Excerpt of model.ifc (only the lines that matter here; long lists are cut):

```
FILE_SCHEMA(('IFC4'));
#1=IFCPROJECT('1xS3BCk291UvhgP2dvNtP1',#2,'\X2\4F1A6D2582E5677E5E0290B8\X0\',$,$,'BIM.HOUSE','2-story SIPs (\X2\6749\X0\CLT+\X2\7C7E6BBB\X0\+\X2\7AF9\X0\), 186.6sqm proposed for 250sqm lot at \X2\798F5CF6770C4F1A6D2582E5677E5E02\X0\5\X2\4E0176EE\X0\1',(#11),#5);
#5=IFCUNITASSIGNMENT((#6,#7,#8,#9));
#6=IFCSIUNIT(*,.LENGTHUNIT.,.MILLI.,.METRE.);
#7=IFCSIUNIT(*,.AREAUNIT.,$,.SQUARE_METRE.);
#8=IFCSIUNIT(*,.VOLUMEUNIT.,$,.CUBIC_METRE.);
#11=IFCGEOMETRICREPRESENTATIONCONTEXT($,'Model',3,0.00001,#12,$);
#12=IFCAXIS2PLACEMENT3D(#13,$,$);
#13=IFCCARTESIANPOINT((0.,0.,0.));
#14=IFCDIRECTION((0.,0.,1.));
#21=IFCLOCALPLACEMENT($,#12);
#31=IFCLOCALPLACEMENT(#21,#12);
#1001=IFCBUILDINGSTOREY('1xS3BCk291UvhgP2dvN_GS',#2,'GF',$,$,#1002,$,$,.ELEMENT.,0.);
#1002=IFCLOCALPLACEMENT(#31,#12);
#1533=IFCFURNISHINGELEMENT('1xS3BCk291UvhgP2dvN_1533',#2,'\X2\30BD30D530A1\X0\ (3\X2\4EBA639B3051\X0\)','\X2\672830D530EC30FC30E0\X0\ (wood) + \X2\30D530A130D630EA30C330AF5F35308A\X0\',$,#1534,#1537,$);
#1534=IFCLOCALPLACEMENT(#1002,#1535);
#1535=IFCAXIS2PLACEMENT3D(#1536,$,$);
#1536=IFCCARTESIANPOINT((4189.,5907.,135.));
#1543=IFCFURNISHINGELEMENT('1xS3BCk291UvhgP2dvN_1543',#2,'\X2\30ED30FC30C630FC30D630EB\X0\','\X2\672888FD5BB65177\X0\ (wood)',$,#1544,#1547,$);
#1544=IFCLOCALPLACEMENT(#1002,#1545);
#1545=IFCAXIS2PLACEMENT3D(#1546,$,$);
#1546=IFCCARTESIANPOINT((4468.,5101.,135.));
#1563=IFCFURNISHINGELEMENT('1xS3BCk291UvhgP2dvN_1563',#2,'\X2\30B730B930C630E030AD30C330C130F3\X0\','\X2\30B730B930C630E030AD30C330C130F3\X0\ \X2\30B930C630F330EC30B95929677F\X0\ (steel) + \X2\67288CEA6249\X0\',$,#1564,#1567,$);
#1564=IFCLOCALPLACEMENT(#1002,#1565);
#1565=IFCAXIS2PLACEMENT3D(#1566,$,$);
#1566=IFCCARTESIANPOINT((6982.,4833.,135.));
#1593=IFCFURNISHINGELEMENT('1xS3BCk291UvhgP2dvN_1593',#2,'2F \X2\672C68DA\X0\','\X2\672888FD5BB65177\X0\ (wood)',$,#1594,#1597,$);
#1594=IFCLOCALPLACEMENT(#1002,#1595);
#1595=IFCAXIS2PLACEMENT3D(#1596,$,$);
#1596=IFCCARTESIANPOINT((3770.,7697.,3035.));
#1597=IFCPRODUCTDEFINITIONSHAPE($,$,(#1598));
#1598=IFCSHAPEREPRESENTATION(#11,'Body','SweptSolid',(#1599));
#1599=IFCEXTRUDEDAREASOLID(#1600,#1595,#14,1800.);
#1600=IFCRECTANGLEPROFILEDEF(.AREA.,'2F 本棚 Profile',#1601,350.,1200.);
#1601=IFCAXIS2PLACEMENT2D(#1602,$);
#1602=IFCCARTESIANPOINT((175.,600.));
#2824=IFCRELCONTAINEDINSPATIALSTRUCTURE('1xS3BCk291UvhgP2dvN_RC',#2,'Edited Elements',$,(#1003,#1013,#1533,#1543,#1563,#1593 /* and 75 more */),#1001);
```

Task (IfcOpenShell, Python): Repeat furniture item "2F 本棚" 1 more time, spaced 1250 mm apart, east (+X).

```python
import numpy as np
import ifcopenshell
import ifcopenshell.api.geometry
import ifcopenshell.api.root
import ifcopenshell.util.element
import ifcopenshell.util.placement
import ifcopenshell.util.unit

model = ifcopenshell.open("model.ifc")
unit_scale = ifcopenshell.util.unit.calculate_unit_scale(model)


def reuse_history(source, copy):
    """copy_class also copies each property set's owner history, people and application; keep the originals."""
    for rel in copy.IsDefinedBy:
        if rel.is_a("IfcRelDefinesByProperties") and (history := rel.RelatingPropertyDefinition.OwnerHistory):
            rel.RelatingPropertyDefinition.OwnerHistory = source.OwnerHistory
            ifcopenshell.util.element.remove_deep2(model, history)


source = model.by_id(1593)
base = ifcopenshell.util.placement.get_local_placement(source.ObjectPlacement)
step = np.array([1.0, 0.0, 0.0]) * 1.25 / unit_scale

for i in range(1, 2):
    copy = ifcopenshell.api.root.copy_class(model, product=source)
    copy.Representation = ifcopenshell.util.element.copy_deep(
        model, source.Representation, exclude=["IfcGeometricRepresentationContext", "IfcRepresentationMap"]
    )
    reuse_history(source, copy)
    matrix = base.copy()
    matrix[:3, 3] += i * step
    print("added at", matrix[:3, 3].round(3) + 0.0)
    ifcopenshell.api.geometry.edit_object_placement(model, product=copy, matrix=matrix, is_si=False)

model.write("model_edited.ifc")
```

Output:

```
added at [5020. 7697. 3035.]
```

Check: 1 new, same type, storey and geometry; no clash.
